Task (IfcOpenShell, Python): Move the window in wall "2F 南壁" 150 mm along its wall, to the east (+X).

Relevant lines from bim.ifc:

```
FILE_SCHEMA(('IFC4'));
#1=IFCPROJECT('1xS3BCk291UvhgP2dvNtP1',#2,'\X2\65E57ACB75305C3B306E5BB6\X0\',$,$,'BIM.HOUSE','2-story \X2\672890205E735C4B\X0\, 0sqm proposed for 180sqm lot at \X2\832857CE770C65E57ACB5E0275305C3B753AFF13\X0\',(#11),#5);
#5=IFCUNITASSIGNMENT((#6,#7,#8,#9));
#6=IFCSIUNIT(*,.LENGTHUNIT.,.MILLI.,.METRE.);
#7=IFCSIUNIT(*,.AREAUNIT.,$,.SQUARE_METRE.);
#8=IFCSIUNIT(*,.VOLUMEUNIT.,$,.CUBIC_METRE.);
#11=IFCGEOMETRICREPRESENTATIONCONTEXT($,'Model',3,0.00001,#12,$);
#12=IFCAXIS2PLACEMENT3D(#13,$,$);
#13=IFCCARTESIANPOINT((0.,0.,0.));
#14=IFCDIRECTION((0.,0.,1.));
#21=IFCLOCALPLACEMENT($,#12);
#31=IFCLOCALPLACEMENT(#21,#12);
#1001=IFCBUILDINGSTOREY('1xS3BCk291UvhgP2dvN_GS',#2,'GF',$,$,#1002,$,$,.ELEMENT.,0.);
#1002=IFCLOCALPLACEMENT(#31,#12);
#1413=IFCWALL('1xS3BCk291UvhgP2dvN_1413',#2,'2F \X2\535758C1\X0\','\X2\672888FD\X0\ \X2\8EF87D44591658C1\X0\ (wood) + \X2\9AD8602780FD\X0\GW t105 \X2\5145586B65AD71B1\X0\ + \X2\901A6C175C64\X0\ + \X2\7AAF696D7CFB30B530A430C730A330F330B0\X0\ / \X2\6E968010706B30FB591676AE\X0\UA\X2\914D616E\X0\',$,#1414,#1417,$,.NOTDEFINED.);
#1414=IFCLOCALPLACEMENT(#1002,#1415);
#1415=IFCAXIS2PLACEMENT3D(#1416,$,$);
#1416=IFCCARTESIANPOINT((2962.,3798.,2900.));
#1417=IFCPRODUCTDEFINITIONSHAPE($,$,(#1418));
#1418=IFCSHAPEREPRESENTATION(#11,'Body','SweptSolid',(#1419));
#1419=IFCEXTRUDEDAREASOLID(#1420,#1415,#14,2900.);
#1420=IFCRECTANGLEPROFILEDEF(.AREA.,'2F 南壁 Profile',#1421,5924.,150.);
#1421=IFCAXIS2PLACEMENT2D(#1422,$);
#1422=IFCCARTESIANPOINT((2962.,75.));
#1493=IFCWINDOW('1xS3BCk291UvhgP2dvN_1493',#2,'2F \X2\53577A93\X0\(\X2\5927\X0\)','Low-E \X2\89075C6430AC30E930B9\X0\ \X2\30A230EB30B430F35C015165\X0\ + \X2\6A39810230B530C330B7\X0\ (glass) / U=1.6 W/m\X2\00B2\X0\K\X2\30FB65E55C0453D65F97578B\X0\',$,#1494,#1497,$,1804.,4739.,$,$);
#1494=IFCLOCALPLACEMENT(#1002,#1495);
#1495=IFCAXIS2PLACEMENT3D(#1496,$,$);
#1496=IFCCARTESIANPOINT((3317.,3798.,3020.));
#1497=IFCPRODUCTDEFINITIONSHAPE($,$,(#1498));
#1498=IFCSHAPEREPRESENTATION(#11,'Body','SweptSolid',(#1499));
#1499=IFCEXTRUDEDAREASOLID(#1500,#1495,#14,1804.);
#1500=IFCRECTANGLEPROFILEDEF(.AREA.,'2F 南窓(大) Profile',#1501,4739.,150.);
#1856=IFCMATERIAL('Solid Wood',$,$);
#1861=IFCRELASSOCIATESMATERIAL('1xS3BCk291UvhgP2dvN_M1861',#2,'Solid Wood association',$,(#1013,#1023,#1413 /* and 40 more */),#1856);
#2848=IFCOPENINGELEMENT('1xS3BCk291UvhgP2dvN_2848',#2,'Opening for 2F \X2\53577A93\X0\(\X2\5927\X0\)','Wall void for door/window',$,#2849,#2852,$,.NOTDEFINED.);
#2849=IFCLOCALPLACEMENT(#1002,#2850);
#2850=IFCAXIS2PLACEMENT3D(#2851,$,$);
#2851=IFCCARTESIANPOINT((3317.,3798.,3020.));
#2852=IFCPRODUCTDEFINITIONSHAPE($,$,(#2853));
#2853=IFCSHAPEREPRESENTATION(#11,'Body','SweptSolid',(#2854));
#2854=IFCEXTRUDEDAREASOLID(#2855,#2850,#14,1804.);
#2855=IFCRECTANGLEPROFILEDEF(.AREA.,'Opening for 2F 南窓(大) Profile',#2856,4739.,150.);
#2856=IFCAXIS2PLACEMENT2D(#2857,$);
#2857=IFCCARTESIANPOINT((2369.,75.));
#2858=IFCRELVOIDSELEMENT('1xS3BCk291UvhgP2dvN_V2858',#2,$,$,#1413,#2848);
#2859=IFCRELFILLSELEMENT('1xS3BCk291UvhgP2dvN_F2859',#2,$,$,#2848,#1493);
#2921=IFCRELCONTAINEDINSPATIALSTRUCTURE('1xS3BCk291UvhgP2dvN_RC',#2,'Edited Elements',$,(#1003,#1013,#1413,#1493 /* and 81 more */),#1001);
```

```python
import ifcopenshell
import ifcopenshell.api.geometry
import ifcopenshell.util.placement

model = ifcopenshell.open("bim.ifc")

window = model.by_guid("1xS3BCk291UvhgP2dvN_1493")
opening = window.FillsVoids[0].RelatingOpeningElement
wall = opening.VoidsElements[0].RelatingBuildingElement

wall_matrix = ifcopenshell.util.placement.get_local_placement(wall.ObjectPlacement)
shift = wall_matrix[:3, 0] * 150.0
before = ifcopenshell.util.placement.get_local_placement(window.ObjectPlacement)[:3, 3].copy()

# The window is not placed relative to its opening, so move both.
for product in (opening, window):
    matrix = ifcopenshell.util.placement.get_local_placement(product.ObjectPlacement)
    matrix[:3, 3] += shift
    ifcopenshell.api.geometry.edit_object_placement(model, product=product, matrix=matrix, is_si=False)

after = ifcopenshell.util.placement.get_local_placement(window.ObjectPlacement)[:3, 3]
print("window moved by", (after - before).round(3) + 0.0)

model.write("bim_v2.ifc")
```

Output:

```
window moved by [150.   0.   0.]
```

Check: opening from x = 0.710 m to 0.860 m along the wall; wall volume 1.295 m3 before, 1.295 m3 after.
